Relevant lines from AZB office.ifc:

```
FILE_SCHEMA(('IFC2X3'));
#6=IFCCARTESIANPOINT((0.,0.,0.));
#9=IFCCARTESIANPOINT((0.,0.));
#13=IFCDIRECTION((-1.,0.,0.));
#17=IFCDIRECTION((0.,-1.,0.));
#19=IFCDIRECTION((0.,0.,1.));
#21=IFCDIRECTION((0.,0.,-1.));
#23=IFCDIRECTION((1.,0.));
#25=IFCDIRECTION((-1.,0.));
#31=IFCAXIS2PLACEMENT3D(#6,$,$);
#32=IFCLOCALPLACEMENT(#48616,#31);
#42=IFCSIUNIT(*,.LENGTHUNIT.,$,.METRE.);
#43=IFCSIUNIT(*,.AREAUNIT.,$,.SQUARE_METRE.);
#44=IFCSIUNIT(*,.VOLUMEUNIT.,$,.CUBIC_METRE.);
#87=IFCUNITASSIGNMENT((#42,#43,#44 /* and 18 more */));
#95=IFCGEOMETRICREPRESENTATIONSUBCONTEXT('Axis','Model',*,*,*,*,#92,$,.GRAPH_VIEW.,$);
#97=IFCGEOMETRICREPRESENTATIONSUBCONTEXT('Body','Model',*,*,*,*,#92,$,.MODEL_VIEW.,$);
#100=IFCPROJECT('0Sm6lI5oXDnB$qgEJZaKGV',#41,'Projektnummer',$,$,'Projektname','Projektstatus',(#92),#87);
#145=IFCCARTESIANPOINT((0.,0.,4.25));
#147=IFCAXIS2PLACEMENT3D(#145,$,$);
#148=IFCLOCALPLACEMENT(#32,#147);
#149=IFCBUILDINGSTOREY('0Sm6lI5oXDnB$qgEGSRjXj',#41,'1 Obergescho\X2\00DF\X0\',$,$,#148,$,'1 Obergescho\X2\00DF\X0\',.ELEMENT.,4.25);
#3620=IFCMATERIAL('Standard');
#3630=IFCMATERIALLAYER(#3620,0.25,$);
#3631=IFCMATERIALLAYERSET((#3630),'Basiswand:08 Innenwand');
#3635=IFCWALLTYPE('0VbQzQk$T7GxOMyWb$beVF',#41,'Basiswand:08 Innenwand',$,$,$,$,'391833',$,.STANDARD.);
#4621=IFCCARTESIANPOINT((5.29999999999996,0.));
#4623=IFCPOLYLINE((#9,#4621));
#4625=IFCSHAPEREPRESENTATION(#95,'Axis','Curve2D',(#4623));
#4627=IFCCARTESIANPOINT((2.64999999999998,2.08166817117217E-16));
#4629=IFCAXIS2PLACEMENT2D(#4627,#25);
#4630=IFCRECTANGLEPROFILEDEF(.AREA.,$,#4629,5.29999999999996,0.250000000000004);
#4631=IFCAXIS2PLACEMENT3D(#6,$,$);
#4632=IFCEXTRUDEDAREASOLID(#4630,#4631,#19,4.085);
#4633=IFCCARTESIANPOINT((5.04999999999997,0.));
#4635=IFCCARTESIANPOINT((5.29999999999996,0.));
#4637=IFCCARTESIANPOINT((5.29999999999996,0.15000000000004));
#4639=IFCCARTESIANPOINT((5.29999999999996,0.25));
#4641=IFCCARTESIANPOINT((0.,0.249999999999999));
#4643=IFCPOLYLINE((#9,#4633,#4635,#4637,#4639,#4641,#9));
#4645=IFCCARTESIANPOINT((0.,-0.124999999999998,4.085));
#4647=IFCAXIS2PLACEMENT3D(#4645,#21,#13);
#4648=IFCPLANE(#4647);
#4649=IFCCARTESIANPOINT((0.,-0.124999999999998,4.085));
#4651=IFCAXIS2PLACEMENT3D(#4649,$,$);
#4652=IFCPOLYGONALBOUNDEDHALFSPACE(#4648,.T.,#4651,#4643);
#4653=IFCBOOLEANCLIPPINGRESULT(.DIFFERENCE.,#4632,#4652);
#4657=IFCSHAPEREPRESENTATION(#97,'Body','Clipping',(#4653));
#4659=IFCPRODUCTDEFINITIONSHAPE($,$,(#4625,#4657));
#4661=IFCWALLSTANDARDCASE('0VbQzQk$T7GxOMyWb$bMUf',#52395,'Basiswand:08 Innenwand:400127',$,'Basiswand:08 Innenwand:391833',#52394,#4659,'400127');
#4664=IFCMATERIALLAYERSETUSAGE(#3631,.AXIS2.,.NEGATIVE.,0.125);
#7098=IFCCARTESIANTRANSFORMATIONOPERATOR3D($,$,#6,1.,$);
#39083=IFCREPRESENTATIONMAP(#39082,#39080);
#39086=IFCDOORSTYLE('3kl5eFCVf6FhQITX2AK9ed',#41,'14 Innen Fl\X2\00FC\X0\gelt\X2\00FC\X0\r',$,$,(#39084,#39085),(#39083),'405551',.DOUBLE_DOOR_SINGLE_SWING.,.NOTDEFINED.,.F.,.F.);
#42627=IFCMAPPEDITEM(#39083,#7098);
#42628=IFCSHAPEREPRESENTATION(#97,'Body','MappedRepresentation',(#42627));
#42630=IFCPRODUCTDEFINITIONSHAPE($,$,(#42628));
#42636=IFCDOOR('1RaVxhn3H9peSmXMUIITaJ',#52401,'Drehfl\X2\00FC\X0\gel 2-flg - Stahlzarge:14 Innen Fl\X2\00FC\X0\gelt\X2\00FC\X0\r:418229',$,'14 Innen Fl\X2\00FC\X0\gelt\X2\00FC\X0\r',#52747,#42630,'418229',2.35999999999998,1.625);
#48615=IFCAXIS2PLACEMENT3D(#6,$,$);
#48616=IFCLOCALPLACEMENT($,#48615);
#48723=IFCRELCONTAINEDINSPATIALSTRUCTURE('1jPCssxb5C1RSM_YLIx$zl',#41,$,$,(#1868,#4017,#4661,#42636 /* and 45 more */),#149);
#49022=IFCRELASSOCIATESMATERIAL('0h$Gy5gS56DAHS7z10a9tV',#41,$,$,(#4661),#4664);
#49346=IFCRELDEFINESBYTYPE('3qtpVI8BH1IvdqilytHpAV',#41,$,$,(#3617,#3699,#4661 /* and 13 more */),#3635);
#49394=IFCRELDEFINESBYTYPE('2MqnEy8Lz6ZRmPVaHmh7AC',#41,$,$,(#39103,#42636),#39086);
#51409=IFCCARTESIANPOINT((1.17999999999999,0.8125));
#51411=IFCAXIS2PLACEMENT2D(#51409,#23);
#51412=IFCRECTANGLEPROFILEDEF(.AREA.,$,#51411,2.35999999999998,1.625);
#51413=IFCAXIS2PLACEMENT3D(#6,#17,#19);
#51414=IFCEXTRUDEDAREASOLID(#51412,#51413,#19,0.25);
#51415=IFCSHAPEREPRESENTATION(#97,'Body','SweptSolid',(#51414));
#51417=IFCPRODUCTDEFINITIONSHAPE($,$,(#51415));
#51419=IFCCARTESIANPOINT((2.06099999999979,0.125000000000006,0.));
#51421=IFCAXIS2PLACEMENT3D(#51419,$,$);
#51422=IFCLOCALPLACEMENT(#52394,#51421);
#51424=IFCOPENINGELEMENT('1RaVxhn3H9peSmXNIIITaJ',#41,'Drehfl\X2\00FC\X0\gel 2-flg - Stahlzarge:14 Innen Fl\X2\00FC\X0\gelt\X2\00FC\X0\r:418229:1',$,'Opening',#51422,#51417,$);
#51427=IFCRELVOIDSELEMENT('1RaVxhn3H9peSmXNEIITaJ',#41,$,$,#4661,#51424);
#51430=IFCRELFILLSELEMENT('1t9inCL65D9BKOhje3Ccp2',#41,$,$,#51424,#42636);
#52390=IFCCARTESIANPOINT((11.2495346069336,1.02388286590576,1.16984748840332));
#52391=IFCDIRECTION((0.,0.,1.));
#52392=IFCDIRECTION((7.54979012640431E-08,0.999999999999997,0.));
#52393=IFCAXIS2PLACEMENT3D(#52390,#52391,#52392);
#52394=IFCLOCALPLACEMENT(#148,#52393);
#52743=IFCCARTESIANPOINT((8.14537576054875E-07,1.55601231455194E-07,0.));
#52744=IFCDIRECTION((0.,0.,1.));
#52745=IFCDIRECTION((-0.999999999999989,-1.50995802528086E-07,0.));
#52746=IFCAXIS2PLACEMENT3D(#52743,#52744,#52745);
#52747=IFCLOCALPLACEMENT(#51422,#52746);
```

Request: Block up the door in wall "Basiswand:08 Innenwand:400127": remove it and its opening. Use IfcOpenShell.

```python
import ifcopenshell
import ifcopenshell.api.feature
import ifcopenshell.api.root
import ifcopenshell.geom
import ifcopenshell.util.shape

model = ifcopenshell.open("AZB office.ifc")
settings = ifcopenshell.geom.settings()


def volume(element):
    """Net volume in cubic metres, openings subtracted."""
    shape = ifcopenshell.geom.create_shape(settings, element)
    return ifcopenshell.util.shape.get_volume(shape.geometry)


door = model.by_id(42636)
opening = door.FillsVoids[0].RelatingOpeningElement
wall = opening.VoidsElements[0].RelatingBuildingElement
before = volume(wall)

ifcopenshell.api.root.remove_product(model, product=door)
ifcopenshell.api.feature.remove_feature(model, feature=opening)

after = volume(wall)

print(f"wall volume {before:.3f} -> {after:.3f} m3")

model.write("AZB office_v2.ifc")
```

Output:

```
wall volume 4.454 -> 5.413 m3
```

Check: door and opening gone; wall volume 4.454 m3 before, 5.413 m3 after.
